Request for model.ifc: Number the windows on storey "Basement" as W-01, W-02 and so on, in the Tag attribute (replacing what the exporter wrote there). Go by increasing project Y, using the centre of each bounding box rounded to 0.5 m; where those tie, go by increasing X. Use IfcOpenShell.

First a look at what the model holds.

```python
import ifcopenshell
import ifcopenshell.util.element
import ifcopenshell.util.placement

model = ifcopenshell.open("model.ifc")
print(model.schema)
storey = next(s for s in model.by_type("IfcBuildingStorey") if s.Name == "Basement")
windows = [e for e in ifcopenshell.util.element.get_decomposition(storey) if e.is_a("IfcWindow")]
for e in sorted(windows, key=lambda e: e.id()):
    origin = ifcopenshell.util.placement.get_local_placement(e.ObjectPlacement)[:3, 3]
    print(e.id(), e.Tag, e.Name, origin.round(2) + 0.0, sep=" | ")
```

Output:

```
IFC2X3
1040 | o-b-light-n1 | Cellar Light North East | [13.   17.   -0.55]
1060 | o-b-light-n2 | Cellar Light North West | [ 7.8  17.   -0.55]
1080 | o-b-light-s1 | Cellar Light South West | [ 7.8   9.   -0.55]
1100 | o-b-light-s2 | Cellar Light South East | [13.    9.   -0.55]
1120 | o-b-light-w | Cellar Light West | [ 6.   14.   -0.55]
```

```python
import ifcopenshell
import ifcopenshell.geom
import ifcopenshell.util.element
import ifcopenshell.util.shape

model = ifcopenshell.open("model.ifc")
settings = ifcopenshell.geom.settings()
settings.set("use-world-coords", True)


def centre(element):
    shape = ifcopenshell.geom.create_shape(settings, element)
    return ifcopenshell.util.shape.get_bbox_centroid(shape.geometry)


storey = next(s for s in model.by_type("IfcBuildingStorey") if s.Name == "Basement")
windows = [e for e in ifcopenshell.util.element.get_decomposition(storey) if e.is_a("IfcWindow")]

# Insertion points can sit at a corner or the storey origin, so sort by the geometry (in metres).
centres = {e: centre(e) for e in windows}
windows.sort(key=lambda e: (round(centres[e][1] / 0.5), centres[e][0]))

for i, e in enumerate(windows, start=1):
    number = f"W-{i:02d}"
    e.Tag = number
    print(e.id(), number)

model.write("model_rev.ifc")
```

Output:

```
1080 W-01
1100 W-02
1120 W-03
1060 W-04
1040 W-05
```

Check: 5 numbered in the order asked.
